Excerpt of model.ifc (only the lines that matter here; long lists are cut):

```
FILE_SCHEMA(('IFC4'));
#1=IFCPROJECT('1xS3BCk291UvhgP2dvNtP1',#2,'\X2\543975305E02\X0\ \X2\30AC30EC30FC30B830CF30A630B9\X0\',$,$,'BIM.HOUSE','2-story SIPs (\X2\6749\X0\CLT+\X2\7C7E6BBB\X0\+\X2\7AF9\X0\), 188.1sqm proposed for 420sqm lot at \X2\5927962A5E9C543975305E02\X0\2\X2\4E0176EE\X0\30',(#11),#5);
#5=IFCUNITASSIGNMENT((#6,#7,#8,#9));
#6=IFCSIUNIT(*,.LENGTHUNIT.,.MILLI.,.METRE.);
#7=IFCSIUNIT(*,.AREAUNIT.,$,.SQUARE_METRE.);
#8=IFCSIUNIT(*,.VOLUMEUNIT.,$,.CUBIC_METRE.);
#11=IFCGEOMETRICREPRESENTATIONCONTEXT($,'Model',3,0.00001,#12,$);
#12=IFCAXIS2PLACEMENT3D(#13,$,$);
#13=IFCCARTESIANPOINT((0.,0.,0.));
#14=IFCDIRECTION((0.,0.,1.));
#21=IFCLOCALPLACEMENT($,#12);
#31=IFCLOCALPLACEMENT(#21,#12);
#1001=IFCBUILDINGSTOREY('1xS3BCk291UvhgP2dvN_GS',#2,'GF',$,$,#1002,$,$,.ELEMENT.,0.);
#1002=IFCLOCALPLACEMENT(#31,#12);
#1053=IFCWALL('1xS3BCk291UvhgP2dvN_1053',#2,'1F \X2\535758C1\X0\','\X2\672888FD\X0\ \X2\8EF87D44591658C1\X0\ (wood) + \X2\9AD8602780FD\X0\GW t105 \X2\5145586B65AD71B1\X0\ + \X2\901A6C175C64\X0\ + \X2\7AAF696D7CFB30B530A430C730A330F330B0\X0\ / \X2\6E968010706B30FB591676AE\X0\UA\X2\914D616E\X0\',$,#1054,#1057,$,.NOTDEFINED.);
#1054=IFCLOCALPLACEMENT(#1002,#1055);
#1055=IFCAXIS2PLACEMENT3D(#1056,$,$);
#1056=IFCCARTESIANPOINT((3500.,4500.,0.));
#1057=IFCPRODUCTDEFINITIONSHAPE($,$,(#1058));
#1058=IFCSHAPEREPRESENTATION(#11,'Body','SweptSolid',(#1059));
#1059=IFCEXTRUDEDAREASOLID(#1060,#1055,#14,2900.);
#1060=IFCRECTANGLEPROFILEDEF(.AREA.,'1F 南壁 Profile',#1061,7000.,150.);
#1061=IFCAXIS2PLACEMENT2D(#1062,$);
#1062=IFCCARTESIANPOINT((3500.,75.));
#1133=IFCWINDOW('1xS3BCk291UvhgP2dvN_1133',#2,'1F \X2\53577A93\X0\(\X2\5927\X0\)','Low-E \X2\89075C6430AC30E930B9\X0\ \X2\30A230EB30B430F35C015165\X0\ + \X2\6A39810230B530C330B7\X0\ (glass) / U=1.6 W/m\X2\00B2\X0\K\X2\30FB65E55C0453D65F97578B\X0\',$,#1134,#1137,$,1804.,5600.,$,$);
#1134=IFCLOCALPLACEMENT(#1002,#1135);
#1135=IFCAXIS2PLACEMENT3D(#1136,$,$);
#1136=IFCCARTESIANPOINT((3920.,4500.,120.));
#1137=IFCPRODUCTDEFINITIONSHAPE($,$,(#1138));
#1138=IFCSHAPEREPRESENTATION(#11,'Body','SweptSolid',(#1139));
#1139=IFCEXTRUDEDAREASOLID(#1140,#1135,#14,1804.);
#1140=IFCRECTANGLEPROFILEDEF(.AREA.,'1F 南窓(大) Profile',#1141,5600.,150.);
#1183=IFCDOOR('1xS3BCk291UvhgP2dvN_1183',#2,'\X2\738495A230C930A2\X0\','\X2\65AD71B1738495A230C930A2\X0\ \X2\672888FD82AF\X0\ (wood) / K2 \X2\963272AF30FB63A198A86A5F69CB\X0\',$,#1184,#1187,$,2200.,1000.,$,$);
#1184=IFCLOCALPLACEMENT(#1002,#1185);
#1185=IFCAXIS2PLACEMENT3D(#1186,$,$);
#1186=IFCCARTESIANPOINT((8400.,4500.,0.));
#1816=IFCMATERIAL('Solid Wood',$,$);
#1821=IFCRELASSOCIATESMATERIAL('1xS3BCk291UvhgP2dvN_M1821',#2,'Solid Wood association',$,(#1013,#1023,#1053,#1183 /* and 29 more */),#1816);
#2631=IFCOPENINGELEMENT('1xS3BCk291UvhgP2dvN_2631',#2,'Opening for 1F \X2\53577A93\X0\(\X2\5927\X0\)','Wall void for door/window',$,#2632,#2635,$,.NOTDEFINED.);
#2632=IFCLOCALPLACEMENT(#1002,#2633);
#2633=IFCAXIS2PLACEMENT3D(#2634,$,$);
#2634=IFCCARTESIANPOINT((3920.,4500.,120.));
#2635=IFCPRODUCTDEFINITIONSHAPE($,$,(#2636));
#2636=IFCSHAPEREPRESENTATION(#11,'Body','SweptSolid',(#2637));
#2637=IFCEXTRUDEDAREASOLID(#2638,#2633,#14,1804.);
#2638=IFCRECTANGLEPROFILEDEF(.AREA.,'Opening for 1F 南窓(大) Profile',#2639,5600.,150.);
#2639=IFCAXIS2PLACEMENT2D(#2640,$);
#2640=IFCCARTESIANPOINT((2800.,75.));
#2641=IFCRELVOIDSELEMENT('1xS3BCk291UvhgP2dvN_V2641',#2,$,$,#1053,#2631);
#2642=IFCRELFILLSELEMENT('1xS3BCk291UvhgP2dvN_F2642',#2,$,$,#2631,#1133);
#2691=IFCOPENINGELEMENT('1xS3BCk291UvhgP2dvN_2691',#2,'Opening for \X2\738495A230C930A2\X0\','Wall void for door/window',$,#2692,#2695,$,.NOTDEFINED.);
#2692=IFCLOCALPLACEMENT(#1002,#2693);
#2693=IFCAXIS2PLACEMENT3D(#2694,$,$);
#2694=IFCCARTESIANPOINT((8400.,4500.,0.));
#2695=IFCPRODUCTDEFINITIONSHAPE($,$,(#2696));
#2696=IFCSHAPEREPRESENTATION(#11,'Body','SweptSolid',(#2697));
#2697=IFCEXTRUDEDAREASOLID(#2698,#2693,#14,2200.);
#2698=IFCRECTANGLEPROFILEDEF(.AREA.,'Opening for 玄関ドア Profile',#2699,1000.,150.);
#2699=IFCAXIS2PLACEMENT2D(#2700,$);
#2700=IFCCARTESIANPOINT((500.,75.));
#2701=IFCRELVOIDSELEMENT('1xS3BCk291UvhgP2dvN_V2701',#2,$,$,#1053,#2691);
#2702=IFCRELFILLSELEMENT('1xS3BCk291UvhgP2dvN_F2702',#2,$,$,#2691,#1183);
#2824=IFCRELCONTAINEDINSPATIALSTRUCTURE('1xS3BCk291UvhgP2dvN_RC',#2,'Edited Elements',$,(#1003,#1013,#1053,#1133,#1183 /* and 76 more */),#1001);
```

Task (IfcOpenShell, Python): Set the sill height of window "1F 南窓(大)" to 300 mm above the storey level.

```python
import numpy as np
import ifcopenshell
import ifcopenshell.api.geometry
import ifcopenshell.geom
import ifcopenshell.util.element
import ifcopenshell.util.placement
import ifcopenshell.util.shape
import ifcopenshell.util.unit

model = ifcopenshell.open("model.ifc")
unit_scale = ifcopenshell.util.unit.calculate_unit_scale(model)

window = model.by_guid("1xS3BCk291UvhgP2dvN_1133")
opening = window.FillsVoids[0].RelatingOpeningElement
storey = ifcopenshell.util.element.get_container(window, ifc_class="IfcBuildingStorey")
level = ifcopenshell.util.placement.get_local_placement(storey.ObjectPlacement)[2, 3]

# The opening's origin need not be at the sill, so measure its lowest point.
shape = ifcopenshell.geom.create_shape(ifcopenshell.geom.settings(), opening)
bottom = ifcopenshell.util.shape.get_shape_bottom_elevation(shape, shape.geometry) / unit_scale
dz = level + 0.3 / unit_scale - bottom

shift = np.array([0.0, 0.0, dz])
# The window is not placed relative to its opening, so move both.
for product in (opening, window):
    matrix = ifcopenshell.util.placement.get_local_placement(product.ObjectPlacement)
    matrix[:3, 3] += shift
    ifcopenshell.api.geometry.edit_object_placement(model, product=product, matrix=matrix, is_si=False)

print(f"moved by {dz * unit_scale:+.3f} m")

model.write("model_edited.ifc")
```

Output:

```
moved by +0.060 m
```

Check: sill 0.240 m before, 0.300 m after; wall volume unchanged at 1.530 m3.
